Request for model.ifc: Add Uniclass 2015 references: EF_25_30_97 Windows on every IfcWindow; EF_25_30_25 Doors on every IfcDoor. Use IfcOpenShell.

First a look at what the model holds.

```python
import ifcopenshell

model = ifcopenshell.open("model.ifc")
print(model.schema)
print("classifications:", [c.Name for c in model.by_type("IfcClassification")])
for ifc_class in ("IfcDoor", "IfcRoof", "IfcStair", "IfcWall", "IfcWindow"):
    print(ifc_class, len(model.by_type(ifc_class)))
```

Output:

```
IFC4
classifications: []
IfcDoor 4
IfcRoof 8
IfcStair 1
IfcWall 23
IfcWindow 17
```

```python
import ifcopenshell
import ifcopenshell.api.classification

model = ifcopenshell.open("model.ifc")

system = ifcopenshell.api.classification.add_classification(model, classification="Uniclass 2015")

codes = {
    "IfcWindow": ("EF_25_30_97", "Windows"),
    "IfcDoor": ("EF_25_30_25", "Doors"),
}
for ifc_class, (code, name) in codes.items():
    products = model.by_type(ifc_class)
    ifcopenshell.api.classification.add_reference(
        model, products=products, classification=system, identification=code, name=name
    )
    print(code, len(products))

model.write("model-out.ifc")
```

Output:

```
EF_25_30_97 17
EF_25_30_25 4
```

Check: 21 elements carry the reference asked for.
